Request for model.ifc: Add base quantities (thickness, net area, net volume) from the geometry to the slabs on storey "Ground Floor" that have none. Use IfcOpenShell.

First a look at what the model holds.

```python
import ifcopenshell
import ifcopenshell.util.element
import ifcopenshell.util.unit

model = ifcopenshell.open("model.ifc")
print(model.schema)
for unit_type in ("LENGTHUNIT", "AREAUNIT", "VOLUMEUNIT"):
    print(unit_type, ifcopenshell.util.unit.calculate_unit_scale(model, unit_type))
storey = next(s for s in model.by_type("IfcBuildingStorey") if s.Name == "Ground Floor")
slabs = [e for e in ifcopenshell.util.element.get_decomposition(storey) if e.is_a("IfcSlab")]
for e in sorted(slabs, key=lambda e: e.id()):
    print(e.id(), e.is_a(), e.Name, list(ifcopenshell.util.element.get_psets(e, qtos_only=True)), sep=" | ")
```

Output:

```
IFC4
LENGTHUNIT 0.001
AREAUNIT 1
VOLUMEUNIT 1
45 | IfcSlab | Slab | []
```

```python
import ifcopenshell
import ifcopenshell.api.pset
import ifcopenshell.geom
import ifcopenshell.util.element
import ifcopenshell.util.shape
import ifcopenshell.util.unit

model = ifcopenshell.open("model.ifc")
unit_scale = ifcopenshell.util.unit.calculate_unit_scale(model)
area_scale = ifcopenshell.util.unit.calculate_unit_scale(model, "AREAUNIT")
volume_scale = ifcopenshell.util.unit.calculate_unit_scale(model, "VOLUMEUNIT")
settings = ifcopenshell.geom.settings()

storey = next(s for s in model.by_type("IfcBuildingStorey") if s.Name == "Ground Floor")
slabs = [e for e in ifcopenshell.util.element.get_decomposition(storey) if e.is_a("IfcSlab")]

for e in sorted(slabs, key=lambda e: e.id()):
    if ifcopenshell.util.element.get_psets(e, qtos_only=True, should_inherit=False):
        continue
    # Geometry comes back in metres, in the element's own axes.
    shape = ifcopenshell.geom.create_shape(settings, e)
    values = {
        "Width": ifcopenshell.util.shape.get_z(shape.geometry) / unit_scale,
        "NetArea": ifcopenshell.util.shape.get_footprint_area(shape.geometry) / area_scale,
        "NetVolume": ifcopenshell.util.shape.get_volume(shape.geometry) / volume_scale,
    }
    qto = ifcopenshell.api.pset.add_qto(model, product=e, name="Qto_SlabBaseQuantities")
    ifcopenshell.api.pset.edit_qto(model, qto=qto, properties=values)
    print(e.id(), {k: round(v, 3) for k, v in values.items()})

model.write("model_v2.ifc")
```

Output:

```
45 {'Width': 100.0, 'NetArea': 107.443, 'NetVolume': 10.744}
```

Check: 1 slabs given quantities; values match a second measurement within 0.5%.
